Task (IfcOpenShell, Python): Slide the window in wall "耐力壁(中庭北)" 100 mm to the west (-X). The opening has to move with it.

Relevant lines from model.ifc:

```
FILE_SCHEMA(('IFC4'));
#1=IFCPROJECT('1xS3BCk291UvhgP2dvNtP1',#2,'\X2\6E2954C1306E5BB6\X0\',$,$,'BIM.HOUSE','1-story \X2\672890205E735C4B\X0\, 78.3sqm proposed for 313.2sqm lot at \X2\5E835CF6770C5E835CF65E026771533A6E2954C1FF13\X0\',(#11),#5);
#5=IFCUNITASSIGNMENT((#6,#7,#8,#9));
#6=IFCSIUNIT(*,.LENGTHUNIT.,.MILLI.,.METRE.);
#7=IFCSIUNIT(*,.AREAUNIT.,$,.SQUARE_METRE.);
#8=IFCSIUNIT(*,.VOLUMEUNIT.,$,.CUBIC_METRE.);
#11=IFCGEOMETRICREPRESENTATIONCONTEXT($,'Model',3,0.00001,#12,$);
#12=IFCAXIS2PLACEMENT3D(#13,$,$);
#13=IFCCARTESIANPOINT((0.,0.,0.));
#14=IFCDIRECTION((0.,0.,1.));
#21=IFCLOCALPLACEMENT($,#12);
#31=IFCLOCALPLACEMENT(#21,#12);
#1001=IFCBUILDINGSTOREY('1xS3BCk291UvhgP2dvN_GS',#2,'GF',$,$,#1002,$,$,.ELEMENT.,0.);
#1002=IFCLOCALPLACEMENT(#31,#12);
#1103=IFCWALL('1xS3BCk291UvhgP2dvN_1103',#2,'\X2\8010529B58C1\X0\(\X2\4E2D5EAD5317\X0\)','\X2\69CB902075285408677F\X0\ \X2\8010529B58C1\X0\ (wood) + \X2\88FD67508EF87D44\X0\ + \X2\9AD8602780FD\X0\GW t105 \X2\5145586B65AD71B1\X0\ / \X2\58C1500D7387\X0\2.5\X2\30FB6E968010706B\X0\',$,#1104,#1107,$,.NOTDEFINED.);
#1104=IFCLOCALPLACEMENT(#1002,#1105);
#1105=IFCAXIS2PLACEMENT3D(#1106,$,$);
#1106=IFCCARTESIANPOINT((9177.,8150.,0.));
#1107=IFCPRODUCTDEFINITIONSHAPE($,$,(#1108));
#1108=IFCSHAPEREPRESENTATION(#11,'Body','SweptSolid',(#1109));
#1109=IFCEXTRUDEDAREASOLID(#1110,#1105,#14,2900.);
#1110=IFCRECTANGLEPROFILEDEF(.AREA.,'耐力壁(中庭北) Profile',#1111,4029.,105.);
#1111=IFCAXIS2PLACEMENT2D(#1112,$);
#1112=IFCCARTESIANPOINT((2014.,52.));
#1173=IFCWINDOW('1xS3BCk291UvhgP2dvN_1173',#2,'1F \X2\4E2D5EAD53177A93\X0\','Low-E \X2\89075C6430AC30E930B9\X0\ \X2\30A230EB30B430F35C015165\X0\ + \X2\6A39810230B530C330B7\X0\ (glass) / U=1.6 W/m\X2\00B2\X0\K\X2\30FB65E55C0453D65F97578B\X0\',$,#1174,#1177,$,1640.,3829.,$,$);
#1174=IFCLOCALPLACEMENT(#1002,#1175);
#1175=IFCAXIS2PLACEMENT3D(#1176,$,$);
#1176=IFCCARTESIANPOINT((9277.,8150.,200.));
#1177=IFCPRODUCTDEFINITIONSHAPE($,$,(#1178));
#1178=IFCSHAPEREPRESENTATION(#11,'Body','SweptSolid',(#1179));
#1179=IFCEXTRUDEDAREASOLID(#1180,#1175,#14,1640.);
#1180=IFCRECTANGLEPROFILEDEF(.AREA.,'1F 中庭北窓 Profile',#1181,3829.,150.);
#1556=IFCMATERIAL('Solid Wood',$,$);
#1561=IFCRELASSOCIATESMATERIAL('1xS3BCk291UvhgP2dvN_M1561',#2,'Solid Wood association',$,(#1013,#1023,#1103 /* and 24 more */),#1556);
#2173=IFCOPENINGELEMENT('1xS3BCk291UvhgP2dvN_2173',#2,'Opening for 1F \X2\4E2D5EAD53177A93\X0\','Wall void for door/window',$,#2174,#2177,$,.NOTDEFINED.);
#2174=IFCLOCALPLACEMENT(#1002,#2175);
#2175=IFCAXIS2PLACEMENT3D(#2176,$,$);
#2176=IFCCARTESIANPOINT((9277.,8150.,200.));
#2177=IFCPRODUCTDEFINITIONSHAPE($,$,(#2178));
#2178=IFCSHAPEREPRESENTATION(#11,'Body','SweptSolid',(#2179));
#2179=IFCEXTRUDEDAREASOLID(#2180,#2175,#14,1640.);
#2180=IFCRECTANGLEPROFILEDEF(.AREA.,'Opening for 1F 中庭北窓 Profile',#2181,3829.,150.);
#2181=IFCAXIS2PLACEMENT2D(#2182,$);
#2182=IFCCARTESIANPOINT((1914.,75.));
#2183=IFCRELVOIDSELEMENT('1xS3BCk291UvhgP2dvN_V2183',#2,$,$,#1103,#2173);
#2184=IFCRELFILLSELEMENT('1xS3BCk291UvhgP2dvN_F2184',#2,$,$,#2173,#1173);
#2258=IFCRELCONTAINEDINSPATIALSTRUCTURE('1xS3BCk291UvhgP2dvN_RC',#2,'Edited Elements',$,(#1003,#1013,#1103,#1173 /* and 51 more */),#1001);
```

```python
import ifcopenshell
import ifcopenshell.api.geometry
import ifcopenshell.util.placement

model = ifcopenshell.open("model.ifc")

window = model.by_guid("1xS3BCk291UvhgP2dvN_1173")
opening = window.FillsVoids[0].RelatingOpeningElement
wall = opening.VoidsElements[0].RelatingBuildingElement

wall_matrix = ifcopenshell.util.placement.get_local_placement(wall.ObjectPlacement)
shift = wall_matrix[:3, 0] * -100.0
before = ifcopenshell.util.placement.get_local_placement(window.ObjectPlacement)[:3, 3].copy()

# The window is not placed relative to its opening, so move both.
for product in (opening, window):
    matrix = ifcopenshell.util.placement.get_local_placement(product.ObjectPlacement)
    matrix[:3, 3] += shift
    ifcopenshell.api.geometry.edit_object_placement(model, product=product, matrix=matrix, is_si=False)

after = ifcopenshell.util.placement.get_local_placement(window.ObjectPlacement)[:3, 3]
print("window moved by", (after - before).round(3) + 0.0)

model.write("model_rev.ifc")
```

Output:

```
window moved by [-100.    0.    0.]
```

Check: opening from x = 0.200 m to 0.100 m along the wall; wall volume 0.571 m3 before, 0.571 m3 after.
